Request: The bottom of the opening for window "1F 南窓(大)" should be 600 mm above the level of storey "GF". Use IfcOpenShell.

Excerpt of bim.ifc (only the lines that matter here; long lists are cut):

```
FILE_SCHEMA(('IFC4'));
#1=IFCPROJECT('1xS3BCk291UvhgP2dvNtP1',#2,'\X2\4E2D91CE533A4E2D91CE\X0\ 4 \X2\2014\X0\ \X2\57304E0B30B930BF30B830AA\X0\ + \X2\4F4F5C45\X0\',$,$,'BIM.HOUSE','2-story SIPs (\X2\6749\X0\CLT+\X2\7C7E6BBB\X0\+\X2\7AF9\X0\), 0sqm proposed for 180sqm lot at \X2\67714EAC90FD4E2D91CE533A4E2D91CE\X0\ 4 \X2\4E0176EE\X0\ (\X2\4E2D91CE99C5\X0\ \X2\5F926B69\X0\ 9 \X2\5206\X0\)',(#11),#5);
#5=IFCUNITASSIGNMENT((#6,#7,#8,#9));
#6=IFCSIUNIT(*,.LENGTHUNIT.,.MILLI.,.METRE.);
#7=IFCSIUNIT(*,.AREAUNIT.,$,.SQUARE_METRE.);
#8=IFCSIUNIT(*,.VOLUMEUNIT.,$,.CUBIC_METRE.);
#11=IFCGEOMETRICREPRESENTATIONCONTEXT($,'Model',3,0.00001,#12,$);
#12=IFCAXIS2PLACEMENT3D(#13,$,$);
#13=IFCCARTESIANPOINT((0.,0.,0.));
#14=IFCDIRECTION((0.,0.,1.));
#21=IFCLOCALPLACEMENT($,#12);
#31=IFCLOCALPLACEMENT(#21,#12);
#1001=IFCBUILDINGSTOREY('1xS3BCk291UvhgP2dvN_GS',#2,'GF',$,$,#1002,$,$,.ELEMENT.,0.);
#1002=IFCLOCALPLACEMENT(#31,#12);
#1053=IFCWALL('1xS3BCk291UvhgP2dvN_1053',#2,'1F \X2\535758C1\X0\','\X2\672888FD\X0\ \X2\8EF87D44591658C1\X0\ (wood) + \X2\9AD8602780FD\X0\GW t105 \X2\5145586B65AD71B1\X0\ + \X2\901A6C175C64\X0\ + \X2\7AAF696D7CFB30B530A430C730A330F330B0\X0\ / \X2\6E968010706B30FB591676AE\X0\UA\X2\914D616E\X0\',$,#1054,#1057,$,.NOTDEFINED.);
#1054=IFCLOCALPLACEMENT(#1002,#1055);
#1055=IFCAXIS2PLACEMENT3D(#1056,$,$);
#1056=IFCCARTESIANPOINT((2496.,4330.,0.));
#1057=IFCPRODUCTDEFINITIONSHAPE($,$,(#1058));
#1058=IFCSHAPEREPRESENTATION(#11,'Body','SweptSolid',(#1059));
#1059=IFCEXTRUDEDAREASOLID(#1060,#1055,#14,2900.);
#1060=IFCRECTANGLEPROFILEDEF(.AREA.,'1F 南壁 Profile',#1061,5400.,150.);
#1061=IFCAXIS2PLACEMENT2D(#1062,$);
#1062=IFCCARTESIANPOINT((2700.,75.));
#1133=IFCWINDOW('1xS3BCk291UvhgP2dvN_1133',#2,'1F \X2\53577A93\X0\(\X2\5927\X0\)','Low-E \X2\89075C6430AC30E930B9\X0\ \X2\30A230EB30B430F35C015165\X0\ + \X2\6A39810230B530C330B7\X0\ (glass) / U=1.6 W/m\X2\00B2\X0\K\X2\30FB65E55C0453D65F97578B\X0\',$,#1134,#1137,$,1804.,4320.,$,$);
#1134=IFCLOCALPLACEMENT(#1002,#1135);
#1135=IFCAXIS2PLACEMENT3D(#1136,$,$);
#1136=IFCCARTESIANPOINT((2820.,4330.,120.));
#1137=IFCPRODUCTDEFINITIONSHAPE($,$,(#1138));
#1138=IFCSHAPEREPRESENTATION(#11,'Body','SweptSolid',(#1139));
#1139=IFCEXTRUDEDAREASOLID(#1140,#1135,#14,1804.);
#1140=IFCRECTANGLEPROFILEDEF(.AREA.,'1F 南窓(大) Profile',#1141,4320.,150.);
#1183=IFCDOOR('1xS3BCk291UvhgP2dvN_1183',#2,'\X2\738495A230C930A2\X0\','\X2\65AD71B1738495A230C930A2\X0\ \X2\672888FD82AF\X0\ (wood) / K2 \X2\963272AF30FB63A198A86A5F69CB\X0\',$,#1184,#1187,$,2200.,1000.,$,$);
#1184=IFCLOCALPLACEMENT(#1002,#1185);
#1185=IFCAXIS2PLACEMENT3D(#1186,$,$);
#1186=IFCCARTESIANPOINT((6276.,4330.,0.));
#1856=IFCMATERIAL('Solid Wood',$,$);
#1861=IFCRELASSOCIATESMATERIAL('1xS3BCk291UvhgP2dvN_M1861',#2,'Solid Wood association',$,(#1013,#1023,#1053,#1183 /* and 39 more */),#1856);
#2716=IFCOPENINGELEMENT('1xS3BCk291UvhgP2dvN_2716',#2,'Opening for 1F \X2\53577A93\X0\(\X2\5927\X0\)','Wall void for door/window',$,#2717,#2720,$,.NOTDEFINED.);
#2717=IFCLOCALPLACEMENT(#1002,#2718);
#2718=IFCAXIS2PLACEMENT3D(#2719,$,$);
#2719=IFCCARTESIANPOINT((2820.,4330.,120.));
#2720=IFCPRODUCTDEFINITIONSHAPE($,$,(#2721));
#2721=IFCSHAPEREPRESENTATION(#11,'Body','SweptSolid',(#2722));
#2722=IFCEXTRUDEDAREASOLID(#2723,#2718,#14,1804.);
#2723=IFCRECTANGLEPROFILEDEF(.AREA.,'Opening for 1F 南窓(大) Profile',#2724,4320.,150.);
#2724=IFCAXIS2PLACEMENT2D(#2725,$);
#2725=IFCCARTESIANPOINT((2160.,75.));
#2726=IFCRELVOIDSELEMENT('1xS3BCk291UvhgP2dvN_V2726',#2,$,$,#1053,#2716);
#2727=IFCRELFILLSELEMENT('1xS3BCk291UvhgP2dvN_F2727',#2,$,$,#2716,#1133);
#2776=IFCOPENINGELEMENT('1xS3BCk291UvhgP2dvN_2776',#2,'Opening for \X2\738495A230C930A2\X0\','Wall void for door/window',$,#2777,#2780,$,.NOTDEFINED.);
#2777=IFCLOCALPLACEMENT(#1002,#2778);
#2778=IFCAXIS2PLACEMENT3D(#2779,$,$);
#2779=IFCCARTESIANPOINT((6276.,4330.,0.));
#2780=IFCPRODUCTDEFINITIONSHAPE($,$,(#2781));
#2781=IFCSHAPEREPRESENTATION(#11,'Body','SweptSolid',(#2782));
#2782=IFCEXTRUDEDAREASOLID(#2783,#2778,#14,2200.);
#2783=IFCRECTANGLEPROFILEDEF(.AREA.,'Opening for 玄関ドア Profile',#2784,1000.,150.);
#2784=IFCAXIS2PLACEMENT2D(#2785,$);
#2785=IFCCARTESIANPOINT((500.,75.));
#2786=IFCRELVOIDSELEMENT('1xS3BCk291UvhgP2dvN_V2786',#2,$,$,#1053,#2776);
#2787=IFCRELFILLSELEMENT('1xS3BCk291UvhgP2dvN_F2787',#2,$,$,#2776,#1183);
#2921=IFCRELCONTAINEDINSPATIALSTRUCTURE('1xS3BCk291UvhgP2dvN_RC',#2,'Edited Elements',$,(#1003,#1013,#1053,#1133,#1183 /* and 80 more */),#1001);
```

```python
import numpy as np
import ifcopenshell
import ifcopenshell.api.geometry
import ifcopenshell.geom
import ifcopenshell.util.element
import ifcopenshell.util.placement
import ifcopenshell.util.shape
import ifcopenshell.util.unit

model = ifcopenshell.open("bim.ifc")
unit_scale = ifcopenshell.util.unit.calculate_unit_scale(model)

window = model.by_guid("1xS3BCk291UvhgP2dvN_1133")
opening = window.FillsVoids[0].RelatingOpeningElement
storey = ifcopenshell.util.element.get_container(window, ifc_class="IfcBuildingStorey")
level = ifcopenshell.util.placement.get_local_placement(storey.ObjectPlacement)[2, 3]

# The opening's origin need not be at the sill, so measure its lowest point.
shape = ifcopenshell.geom.create_shape(ifcopenshell.geom.settings(), opening)
bottom = ifcopenshell.util.shape.get_shape_bottom_elevation(shape, shape.geometry) / unit_scale
dz = level + 0.6 / unit_scale - bottom

shift = np.array([0.0, 0.0, dz])
# The window is not placed relative to its opening, so move both.
for product in (opening, window):
    matrix = ifcopenshell.util.placement.get_local_placement(product.ObjectPlacement)
    matrix[:3, 3] += shift
    ifcopenshell.api.geometry.edit_object_placement(model, product=product, matrix=matrix, is_si=False)

print(f"moved by {dz * unit_scale:+.3f} m")

model.write("bim_edited.ifc")
```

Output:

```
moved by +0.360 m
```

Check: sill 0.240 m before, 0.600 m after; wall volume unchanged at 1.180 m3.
